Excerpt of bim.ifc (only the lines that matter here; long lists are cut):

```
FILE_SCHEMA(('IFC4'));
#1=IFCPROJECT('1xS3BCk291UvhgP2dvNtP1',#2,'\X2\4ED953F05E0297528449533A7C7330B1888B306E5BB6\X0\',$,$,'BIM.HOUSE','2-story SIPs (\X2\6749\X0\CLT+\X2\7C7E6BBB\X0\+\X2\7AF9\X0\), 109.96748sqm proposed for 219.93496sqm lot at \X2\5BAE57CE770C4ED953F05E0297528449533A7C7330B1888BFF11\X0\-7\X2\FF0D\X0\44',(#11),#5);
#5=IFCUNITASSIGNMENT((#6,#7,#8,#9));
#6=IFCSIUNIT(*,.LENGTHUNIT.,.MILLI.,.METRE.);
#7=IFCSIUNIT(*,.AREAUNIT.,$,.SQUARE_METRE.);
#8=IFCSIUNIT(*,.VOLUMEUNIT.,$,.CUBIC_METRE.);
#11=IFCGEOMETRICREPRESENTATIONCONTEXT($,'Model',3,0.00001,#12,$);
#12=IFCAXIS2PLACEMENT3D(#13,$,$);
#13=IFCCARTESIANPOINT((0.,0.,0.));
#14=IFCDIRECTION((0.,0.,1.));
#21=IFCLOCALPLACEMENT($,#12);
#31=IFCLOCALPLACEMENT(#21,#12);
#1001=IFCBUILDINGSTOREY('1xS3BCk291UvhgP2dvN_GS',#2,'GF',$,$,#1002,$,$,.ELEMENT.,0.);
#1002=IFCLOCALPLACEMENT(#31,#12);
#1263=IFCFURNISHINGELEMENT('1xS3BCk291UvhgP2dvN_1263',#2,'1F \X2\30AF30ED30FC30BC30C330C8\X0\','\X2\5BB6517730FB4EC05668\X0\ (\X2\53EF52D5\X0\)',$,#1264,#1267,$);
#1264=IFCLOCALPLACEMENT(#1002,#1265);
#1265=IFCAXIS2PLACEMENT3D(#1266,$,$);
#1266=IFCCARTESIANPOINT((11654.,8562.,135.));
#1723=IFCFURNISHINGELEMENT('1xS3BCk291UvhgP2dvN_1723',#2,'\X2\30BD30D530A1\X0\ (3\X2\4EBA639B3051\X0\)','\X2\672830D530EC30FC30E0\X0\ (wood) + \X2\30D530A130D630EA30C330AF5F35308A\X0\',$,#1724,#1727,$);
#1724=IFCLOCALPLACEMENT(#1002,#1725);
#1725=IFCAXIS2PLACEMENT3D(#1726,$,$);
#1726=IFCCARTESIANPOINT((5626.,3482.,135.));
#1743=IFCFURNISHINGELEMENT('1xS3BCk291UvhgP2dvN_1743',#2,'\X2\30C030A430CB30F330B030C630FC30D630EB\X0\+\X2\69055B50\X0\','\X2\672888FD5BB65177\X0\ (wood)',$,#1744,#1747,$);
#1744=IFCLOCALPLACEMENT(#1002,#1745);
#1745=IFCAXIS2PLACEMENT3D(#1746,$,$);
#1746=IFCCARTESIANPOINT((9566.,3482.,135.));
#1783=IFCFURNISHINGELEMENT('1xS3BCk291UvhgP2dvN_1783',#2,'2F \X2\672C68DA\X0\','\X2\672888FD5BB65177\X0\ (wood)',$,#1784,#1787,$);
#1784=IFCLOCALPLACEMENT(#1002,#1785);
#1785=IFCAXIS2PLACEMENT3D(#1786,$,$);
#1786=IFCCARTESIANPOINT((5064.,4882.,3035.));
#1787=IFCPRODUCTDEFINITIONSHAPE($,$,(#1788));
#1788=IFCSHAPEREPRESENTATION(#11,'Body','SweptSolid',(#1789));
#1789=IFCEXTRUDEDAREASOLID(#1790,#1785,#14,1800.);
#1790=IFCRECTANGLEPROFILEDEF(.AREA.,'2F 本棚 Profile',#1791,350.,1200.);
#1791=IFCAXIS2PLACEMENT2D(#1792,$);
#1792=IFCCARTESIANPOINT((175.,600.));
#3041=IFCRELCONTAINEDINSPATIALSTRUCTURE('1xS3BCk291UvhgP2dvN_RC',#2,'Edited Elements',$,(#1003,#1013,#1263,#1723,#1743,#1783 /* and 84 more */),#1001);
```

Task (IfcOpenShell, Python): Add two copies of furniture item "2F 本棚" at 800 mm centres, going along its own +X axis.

```python
import ifcopenshell
import ifcopenshell.api.geometry
import ifcopenshell.api.root
import ifcopenshell.util.element
import ifcopenshell.util.placement
import ifcopenshell.util.unit

model = ifcopenshell.open("bim.ifc")
unit_scale = ifcopenshell.util.unit.calculate_unit_scale(model)


def reuse_history(source, copy):
    """copy_class also copies each property set's owner history, people and application; keep the originals."""
    for rel in copy.IsDefinedBy:
        if rel.is_a("IfcRelDefinesByProperties") and (history := rel.RelatingPropertyDefinition.OwnerHistory):
            rel.RelatingPropertyDefinition.OwnerHistory = source.OwnerHistory
            ifcopenshell.util.element.remove_deep2(model, history)


source = model.by_guid("1xS3BCk291UvhgP2dvN_1783")
base = ifcopenshell.util.placement.get_local_placement(source.ObjectPlacement)
step = base[:3, 0] * 0.8 / unit_scale

for i in range(1, 3):
    copy = ifcopenshell.api.root.copy_class(model, product=source)
    copy.Representation = ifcopenshell.util.element.copy_deep(
        model, source.Representation, exclude=["IfcGeometricRepresentationContext", "IfcRepresentationMap"]
    )
    reuse_history(source, copy)
    matrix = base.copy()
    matrix[:3, 3] += i * step
    print("added at", matrix[:3, 3].round(3) + 0.0)
    ifcopenshell.api.geometry.edit_object_placement(model, product=copy, matrix=matrix, is_si=False)

model.write("bim-out.ifc")
```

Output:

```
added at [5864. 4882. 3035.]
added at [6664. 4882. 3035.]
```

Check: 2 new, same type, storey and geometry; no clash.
